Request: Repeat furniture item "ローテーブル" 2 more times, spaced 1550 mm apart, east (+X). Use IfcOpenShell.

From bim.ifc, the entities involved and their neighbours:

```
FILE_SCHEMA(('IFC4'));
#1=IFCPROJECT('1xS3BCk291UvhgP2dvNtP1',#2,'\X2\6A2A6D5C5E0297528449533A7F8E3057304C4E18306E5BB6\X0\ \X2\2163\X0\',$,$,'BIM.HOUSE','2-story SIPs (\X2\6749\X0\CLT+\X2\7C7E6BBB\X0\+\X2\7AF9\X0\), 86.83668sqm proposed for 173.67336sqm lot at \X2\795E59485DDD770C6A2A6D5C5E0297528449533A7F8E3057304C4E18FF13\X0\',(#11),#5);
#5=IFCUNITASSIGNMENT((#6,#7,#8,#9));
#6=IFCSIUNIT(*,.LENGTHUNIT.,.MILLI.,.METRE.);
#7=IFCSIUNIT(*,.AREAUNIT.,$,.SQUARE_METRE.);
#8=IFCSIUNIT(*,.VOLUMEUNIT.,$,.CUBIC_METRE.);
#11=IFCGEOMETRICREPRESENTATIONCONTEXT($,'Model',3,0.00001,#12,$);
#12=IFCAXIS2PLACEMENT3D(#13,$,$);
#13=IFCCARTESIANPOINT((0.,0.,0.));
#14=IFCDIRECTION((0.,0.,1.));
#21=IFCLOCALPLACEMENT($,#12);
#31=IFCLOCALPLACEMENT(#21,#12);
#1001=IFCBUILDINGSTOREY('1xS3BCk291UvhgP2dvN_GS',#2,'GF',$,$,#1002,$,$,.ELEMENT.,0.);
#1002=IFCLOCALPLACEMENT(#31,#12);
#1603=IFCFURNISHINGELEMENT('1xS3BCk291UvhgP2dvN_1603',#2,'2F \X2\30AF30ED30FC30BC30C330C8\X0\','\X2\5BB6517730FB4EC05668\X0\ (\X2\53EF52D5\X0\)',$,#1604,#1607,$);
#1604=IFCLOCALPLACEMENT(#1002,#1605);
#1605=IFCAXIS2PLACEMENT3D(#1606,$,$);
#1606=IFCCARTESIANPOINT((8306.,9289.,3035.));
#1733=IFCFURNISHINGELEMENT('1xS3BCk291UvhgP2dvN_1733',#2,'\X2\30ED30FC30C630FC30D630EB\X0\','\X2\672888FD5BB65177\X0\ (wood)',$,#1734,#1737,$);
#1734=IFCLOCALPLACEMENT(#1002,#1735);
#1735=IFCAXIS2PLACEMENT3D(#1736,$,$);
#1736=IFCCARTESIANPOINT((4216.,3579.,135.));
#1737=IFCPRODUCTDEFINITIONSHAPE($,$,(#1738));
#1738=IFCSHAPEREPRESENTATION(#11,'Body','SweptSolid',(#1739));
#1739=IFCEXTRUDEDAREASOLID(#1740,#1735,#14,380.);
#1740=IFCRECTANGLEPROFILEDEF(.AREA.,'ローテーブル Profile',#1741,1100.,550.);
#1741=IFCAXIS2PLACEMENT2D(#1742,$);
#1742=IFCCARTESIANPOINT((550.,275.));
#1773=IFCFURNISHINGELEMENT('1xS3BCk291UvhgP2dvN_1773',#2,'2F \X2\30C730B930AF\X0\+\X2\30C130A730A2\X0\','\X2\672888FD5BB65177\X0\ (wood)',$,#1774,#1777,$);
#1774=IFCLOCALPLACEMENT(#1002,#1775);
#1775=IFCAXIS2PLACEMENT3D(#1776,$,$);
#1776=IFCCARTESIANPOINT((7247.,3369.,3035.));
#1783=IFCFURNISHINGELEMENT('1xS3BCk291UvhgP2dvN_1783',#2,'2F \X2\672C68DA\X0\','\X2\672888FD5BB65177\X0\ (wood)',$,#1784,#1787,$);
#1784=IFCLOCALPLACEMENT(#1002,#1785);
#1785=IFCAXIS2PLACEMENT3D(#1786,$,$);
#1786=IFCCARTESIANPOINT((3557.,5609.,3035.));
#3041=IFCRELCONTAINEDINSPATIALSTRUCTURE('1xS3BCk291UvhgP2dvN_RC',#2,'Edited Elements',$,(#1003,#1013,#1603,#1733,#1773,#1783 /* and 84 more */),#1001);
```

```python
import numpy as np
import ifcopenshell
import ifcopenshell.api.geometry
import ifcopenshell.api.root
import ifcopenshell.util.element
import ifcopenshell.util.placement
import ifcopenshell.util.unit

model = ifcopenshell.open("bim.ifc")
unit_scale = ifcopenshell.util.unit.calculate_unit_scale(model)


def reuse_history(source, copy):
    """copy_class also copies each property set's owner history, people and application; keep the originals."""
    for rel in copy.IsDefinedBy:
        if rel.is_a("IfcRelDefinesByProperties") and (history := rel.RelatingPropertyDefinition.OwnerHistory):
            rel.RelatingPropertyDefinition.OwnerHistory = source.OwnerHistory
            ifcopenshell.util.element.remove_deep2(model, history)


source = model.by_id(1733)
base = ifcopenshell.util.placement.get_local_placement(source.ObjectPlacement)
step = np.array([1.0, 0.0, 0.0]) * 1.55 / unit_scale

for i in range(1, 3):
    copy = ifcopenshell.api.root.copy_class(model, product=source)
    copy.Representation = ifcopenshell.util.element.copy_deep(
        model, source.Representation, exclude=["IfcGeometricRepresentationContext", "IfcRepresentationMap"]
    )
    reuse_history(source, copy)
    matrix = base.copy()
    matrix[:3, 3] += i * step
    print("added at", matrix[:3, 3].round(3) + 0.0)
    ifcopenshell.api.geometry.edit_object_placement(model, product=copy, matrix=matrix, is_si=False)

model.write("bim_rev.ifc")
```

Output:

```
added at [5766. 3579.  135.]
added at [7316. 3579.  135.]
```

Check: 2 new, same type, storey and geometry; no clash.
